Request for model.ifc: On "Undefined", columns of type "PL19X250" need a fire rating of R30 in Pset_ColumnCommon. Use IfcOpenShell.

First a look at what the model holds.

```python
import ifcopenshell
import ifcopenshell.util.element

model = ifcopenshell.open("model.ifc")
print(model.schema)
storey = next(s for s in model.by_type("IfcBuildingStorey") if s.Name == "Undefined")
columns = [e for e in ifcopenshell.util.element.get_decomposition(storey) if e.is_a("IfcColumn")]
seen = {}
for e in columns:
    element_type = ifcopenshell.util.element.get_type(e)
    key = (element_type.Name if element_type != e and element_type else None, ifcopenshell.util.element.get_pset(e, "Pset_ColumnCommon", "FireRating"))
    seen[key] = seen.get(key, 0) + 1
for (name, value), count in sorted(seen.items(), key=str):
    print(count, "x", name, "|", value)
```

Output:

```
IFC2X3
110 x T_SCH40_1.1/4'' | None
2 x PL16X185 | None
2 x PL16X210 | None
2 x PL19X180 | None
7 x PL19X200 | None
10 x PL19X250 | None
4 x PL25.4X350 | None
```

```python
import ifcopenshell
import ifcopenshell.api.pset
import ifcopenshell.util.element

model = ifcopenshell.open("model.ifc")

storey = next(s for s in model.by_type("IfcBuildingStorey") if s.Name == "Undefined")
columns = [e for e in ifcopenshell.util.element.get_decomposition(storey) if e.is_a("IfcColumn")]

count = 0
for e in columns:
    element_type = ifcopenshell.util.element.get_type(e)
    if element_type in (None, e) or element_type.Name != "PL19X250":
        continue
    # add_pset returns the element's existing set when there is one.
    pset = ifcopenshell.api.pset.add_pset(model, product=e, name="Pset_ColumnCommon")
    ifcopenshell.api.pset.edit_pset(model, pset=pset, properties={"FireRating": "R30"})
    count += 1

print(count, "columns updated")

model.write("model_edited.ifc")
```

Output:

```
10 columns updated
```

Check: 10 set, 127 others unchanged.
